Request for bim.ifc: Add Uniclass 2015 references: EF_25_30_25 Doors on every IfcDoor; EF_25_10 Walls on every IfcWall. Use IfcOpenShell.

First a look at what the model holds.

```python
import ifcopenshell

model = ifcopenshell.open("bim.ifc")
print(model.schema)
print("classifications:", [c.Name for c in model.by_type("IfcClassification")])
for ifc_class in ("IfcDoor", "IfcRoof", "IfcStair", "IfcWall", "IfcWindow"):
    print(ifc_class, len(model.by_type(ifc_class)))
```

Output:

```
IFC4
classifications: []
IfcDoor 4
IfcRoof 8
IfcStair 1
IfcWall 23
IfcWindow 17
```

```python
import ifcopenshell
import ifcopenshell.api.classification

model = ifcopenshell.open("bim.ifc")

system = ifcopenshell.api.classification.add_classification(model, classification="Uniclass 2015")

codes = {
    "IfcDoor": ("EF_25_30_25", "Doors"),
    "IfcWall": ("EF_25_10", "Walls"),
}
for ifc_class, (code, name) in codes.items():
    products = model.by_type(ifc_class)
    ifcopenshell.api.classification.add_reference(
        model, products=products, classification=system, identification=code, name=name
    )
    print(code, len(products))

model.write("bim_v2.ifc")
```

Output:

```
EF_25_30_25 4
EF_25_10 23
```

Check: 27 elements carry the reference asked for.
